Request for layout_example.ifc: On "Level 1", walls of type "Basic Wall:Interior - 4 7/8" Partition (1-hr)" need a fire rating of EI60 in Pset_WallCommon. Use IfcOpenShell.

First a look at what the model holds.

```python
import ifcopenshell
import ifcopenshell.util.element

model = ifcopenshell.open("layout_example.ifc")
print(model.schema)
storey = next(s for s in model.by_type("IfcBuildingStorey") if s.Name == "Level 1")
walls = [e for e in ifcopenshell.util.element.get_decomposition(storey) if e.is_a("IfcWall")]
seen = {}
for e in walls:
    element_type = ifcopenshell.util.element.get_type(e)
    key = (element_type.Name if element_type != e and element_type else None, ifcopenshell.util.element.get_pset(e, "Pset_WallCommon", "FireRating"))
    seen[key] = seen.get(key, 0) + 1
for (name, value), count in sorted(seen.items(), key=str):
    print(count, "x", name, "|", value)
```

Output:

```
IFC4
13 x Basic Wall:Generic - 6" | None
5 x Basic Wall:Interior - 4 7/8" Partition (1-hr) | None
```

```python
import ifcopenshell
import ifcopenshell.api.pset
import ifcopenshell.util.element

model = ifcopenshell.open("layout_example.ifc")

storey = next(s for s in model.by_type("IfcBuildingStorey") if s.Name == "Level 1")
walls = [e for e in ifcopenshell.util.element.get_decomposition(storey) if e.is_a("IfcWall")]

count = 0
for e in walls:
    element_type = ifcopenshell.util.element.get_type(e)
    if element_type in (None, e) or element_type.Name != 'Basic Wall:Interior - 4 7/8" Partition (1-hr)':
        continue
    # add_pset returns the element's existing set when there is one.
    pset = ifcopenshell.api.pset.add_pset(model, product=e, name="Pset_WallCommon")
    ifcopenshell.api.pset.edit_pset(model, pset=pset, properties={"FireRating": "EI60"})
    count += 1

print(count, "walls updated")

model.write("layout_example_edited.ifc")
```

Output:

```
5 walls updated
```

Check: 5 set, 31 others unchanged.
